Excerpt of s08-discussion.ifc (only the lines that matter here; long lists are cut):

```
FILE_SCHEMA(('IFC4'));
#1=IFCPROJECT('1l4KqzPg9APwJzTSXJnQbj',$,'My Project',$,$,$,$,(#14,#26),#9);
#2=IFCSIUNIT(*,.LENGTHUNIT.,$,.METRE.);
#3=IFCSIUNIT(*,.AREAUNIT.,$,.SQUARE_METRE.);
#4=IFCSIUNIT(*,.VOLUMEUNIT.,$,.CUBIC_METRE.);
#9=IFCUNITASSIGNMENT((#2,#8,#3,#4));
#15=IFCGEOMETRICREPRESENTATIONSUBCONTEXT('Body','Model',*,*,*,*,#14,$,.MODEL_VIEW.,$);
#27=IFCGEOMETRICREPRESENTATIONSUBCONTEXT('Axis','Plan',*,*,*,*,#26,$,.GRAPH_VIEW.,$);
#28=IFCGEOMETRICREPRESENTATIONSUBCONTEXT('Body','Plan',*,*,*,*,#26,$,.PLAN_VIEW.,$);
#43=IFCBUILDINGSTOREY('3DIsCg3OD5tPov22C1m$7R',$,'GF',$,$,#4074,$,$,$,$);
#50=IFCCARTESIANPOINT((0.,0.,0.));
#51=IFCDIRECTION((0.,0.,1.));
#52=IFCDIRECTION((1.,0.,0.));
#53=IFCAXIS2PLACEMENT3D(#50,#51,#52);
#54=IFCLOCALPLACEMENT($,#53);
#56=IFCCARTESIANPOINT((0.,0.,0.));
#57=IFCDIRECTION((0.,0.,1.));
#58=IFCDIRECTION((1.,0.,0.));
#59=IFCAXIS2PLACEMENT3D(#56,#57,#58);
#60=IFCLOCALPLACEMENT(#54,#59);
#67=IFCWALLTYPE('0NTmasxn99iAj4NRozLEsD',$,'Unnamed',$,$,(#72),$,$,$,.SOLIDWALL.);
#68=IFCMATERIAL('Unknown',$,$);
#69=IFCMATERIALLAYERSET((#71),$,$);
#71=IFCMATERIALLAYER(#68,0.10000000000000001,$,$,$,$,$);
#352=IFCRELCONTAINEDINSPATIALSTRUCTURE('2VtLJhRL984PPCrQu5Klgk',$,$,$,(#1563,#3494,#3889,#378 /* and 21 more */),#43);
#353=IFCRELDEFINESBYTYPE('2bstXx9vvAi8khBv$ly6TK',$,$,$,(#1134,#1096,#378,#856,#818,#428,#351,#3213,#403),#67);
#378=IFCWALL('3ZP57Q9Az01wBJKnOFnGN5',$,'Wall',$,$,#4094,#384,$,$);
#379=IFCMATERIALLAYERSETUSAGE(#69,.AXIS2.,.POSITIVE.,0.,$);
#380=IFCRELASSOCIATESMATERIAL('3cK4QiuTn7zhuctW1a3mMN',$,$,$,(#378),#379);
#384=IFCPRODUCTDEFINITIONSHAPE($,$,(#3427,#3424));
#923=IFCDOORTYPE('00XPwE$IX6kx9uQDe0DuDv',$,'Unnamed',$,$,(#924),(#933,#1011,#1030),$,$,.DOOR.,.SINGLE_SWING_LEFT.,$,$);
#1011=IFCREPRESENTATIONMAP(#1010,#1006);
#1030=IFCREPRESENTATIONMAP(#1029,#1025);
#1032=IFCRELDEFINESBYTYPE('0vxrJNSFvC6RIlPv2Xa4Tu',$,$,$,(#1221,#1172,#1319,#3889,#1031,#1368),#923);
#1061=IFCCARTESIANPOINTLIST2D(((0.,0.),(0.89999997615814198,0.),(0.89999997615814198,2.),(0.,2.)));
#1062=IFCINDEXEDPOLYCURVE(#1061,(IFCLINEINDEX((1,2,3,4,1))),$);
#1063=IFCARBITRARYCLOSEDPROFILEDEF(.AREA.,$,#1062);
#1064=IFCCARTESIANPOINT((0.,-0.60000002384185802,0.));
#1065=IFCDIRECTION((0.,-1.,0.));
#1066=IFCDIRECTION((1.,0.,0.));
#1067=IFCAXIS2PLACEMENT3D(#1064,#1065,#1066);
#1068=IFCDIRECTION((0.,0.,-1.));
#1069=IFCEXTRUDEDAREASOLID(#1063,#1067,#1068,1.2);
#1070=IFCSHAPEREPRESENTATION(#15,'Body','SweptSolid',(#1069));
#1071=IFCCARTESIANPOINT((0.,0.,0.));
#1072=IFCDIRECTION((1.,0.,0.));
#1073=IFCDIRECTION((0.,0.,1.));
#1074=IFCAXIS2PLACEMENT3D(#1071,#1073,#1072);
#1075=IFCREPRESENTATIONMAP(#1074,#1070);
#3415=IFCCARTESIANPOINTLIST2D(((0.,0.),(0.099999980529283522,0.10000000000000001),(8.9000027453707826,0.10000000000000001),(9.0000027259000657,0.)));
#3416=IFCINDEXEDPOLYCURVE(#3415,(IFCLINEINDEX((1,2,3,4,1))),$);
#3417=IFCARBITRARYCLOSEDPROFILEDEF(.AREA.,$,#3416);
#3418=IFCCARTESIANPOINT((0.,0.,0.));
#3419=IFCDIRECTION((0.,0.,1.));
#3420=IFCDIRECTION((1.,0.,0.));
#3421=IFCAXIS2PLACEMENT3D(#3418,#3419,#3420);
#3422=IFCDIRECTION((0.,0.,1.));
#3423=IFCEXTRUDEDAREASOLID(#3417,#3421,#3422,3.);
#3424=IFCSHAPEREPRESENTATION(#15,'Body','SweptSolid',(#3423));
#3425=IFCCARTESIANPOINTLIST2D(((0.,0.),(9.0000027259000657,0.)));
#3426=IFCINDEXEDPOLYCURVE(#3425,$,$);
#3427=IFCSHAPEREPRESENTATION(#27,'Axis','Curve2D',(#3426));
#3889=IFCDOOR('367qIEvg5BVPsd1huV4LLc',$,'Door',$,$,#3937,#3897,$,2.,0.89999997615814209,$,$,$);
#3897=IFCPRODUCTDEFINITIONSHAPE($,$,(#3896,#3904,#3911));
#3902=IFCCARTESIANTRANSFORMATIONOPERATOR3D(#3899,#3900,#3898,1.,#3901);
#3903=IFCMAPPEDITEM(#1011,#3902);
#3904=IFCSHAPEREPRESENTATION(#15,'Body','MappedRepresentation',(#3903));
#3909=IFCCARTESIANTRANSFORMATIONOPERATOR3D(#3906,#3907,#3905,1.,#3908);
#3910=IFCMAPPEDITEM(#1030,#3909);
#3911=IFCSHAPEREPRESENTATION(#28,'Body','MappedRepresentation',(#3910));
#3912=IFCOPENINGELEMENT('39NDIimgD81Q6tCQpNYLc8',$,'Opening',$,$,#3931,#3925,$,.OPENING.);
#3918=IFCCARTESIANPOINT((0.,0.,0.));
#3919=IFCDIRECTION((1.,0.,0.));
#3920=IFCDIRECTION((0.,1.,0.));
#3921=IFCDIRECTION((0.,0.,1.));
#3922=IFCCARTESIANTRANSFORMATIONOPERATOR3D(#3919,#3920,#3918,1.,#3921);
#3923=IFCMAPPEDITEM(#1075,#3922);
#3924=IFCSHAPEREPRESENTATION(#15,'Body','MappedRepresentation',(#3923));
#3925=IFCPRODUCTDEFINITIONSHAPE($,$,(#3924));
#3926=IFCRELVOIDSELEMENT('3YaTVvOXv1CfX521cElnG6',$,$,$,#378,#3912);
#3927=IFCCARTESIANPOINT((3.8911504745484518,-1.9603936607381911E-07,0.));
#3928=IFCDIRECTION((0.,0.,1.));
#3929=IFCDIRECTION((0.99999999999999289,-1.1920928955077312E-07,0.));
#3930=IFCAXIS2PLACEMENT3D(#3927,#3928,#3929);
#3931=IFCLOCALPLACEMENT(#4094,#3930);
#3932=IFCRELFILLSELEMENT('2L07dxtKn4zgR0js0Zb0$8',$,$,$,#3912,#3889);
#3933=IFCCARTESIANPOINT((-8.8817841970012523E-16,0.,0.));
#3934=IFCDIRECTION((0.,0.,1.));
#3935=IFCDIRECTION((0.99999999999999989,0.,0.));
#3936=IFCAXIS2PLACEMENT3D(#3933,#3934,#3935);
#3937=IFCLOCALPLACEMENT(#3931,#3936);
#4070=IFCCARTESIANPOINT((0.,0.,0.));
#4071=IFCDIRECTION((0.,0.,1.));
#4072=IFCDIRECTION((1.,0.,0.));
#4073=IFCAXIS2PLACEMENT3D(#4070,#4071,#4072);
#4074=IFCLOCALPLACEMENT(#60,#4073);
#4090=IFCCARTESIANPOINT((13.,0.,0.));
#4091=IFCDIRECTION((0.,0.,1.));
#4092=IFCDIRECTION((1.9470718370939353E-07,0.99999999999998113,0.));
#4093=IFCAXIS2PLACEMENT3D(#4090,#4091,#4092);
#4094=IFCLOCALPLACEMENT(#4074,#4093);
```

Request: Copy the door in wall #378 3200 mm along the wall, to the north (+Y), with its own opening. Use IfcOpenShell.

```python
import ifcopenshell
import ifcopenshell.api.feature
import ifcopenshell.api.geometry
import ifcopenshell.api.root
import ifcopenshell.geom
import ifcopenshell.util.element
import ifcopenshell.util.placement
import ifcopenshell.util.shape

model = ifcopenshell.open("s08-discussion.ifc")
settings = ifcopenshell.geom.settings()


def volume(element):
    """Net volume in cubic metres, openings subtracted."""
    shape = ifcopenshell.geom.create_shape(settings, element)
    return ifcopenshell.util.shape.get_volume(shape.geometry)


door = model.by_id(3889)
opening = door.FillsVoids[0].RelatingOpeningElement
wall = opening.VoidsElements[0].RelatingBuildingElement
before = volume(wall)
shift = ifcopenshell.util.placement.get_local_placement(wall.ObjectPlacement)[:3, 0] * 3.2

# copy_class copies the void relationship, type, container and properties, but no geometry.
new_opening = ifcopenshell.api.root.copy_class(model, product=opening)
new_opening.Representation = ifcopenshell.util.element.copy_deep(
    model, opening.Representation, exclude=["IfcGeometricRepresentationContext", "IfcRepresentationMap"]
)
new_door = ifcopenshell.api.root.copy_class(model, product=door)
new_door.Representation = ifcopenshell.util.element.copy_deep(
    model, door.Representation, exclude=["IfcGeometricRepresentationContext", "IfcRepresentationMap"]
)
ifcopenshell.api.feature.add_filling(model, opening=new_opening, element=new_door)

for old, new in ((opening, new_opening), (door, new_door)):
    matrix = ifcopenshell.util.placement.get_local_placement(old.ObjectPlacement)
    matrix[:3, 3] += shift
    ifcopenshell.api.geometry.edit_object_placement(model, product=new, matrix=matrix, is_si=False)

after = volume(wall)

print(f"wall volume {before:.3f} -> {after:.3f} m3")

model.write("s08-discussion_v2.ifc")
```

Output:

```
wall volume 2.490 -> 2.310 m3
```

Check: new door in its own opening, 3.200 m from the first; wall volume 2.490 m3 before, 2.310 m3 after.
